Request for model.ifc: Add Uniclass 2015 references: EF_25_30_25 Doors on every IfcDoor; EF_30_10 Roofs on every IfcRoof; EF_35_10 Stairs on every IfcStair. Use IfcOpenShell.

First a look at what the model holds.

```python
import ifcopenshell

model = ifcopenshell.open("model.ifc")
print(model.schema)
print("classifications:", [c.Name for c in model.by_type("IfcClassification")])
for ifc_class in ("IfcDoor", "IfcRoof", "IfcStair", "IfcWall", "IfcWindow"):
    print(ifc_class, len(model.by_type(ifc_class)))
```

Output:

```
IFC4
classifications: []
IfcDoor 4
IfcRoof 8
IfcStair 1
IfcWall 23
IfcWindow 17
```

```python
import ifcopenshell
import ifcopenshell.api.classification

model = ifcopenshell.open("model.ifc")

system = ifcopenshell.api.classification.add_classification(model, classification="Uniclass 2015")

codes = {
    "IfcDoor": ("EF_25_30_25", "Doors"),
    "IfcRoof": ("EF_30_10", "Roofs"),
    "IfcStair": ("EF_35_10", "Stairs"),
}
for ifc_class, (code, name) in codes.items():
    products = model.by_type(ifc_class)
    ifcopenshell.api.classification.add_reference(
        model, products=products, classification=system, identification=code, name=name
    )
    print(code, len(products))

model.write("model_updated.ifc")
```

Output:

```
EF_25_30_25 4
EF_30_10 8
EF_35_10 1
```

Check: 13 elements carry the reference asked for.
